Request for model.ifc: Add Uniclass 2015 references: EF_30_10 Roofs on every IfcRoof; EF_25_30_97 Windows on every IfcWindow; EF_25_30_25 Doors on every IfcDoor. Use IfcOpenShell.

First a look at what the model holds.

```python
import ifcopenshell

model = ifcopenshell.open("model.ifc")
print(model.schema)
print("classifications:", [c.Name for c in model.by_type("IfcClassification")])
for ifc_class in ("IfcDoor", "IfcRoof", "IfcStair", "IfcWall", "IfcWindow"):
    print(ifc_class, len(model.by_type(ifc_class)))
```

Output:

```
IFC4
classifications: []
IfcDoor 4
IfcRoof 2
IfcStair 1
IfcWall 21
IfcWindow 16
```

```python
import ifcopenshell
import ifcopenshell.api.classification

model = ifcopenshell.open("model.ifc")

system = ifcopenshell.api.classification.add_classification(model, classification="Uniclass 2015")

codes = {
    "IfcRoof": ("EF_30_10", "Roofs"),
    "IfcWindow": ("EF_25_30_97", "Windows"),
    "IfcDoor": ("EF_25_30_25", "Doors"),
}
for ifc_class, (code, name) in codes.items():
    products = model.by_type(ifc_class)
    ifcopenshell.api.classification.add_reference(
        model, products=products, classification=system, identification=code, name=name
    )
    print(code, len(products))

model.write("model_rev.ifc")
```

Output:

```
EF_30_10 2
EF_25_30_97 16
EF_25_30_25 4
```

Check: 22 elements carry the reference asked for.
